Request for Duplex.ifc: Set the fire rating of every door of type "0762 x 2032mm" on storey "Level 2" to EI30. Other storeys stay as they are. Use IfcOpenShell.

First a look at what the model holds.

```python
import ifcopenshell
import ifcopenshell.util.element

model = ifcopenshell.open("Duplex.ifc")
print(model.schema)
storey = next(s for s in model.by_type("IfcBuildingStorey") if s.Name == "Level 2")
doors = [e for e in ifcopenshell.util.element.get_decomposition(storey) if e.is_a("IfcDoor")]
seen = {}
for e in doors:
    element_type = ifcopenshell.util.element.get_type(e)
    key = (element_type.Name if element_type != e and element_type else None, ifcopenshell.util.element.get_pset(e, "Pset_DoorCommon", "FireRating"))
    seen[key] = seen.get(key, 0) + 1
for (name, value), count in sorted(seen.items(), key=str):
    print(count, "x", name, "|", value)
```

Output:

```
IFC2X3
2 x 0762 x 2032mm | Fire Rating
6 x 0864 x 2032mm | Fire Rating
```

```python
import ifcopenshell
import ifcopenshell.api.pset
import ifcopenshell.util.element

model = ifcopenshell.open("Duplex.ifc")

storey = next(s for s in model.by_type("IfcBuildingStorey") if s.Name == "Level 2")
doors = [e for e in ifcopenshell.util.element.get_decomposition(storey) if e.is_a("IfcDoor")]

count = 0
for e in doors:
    element_type = ifcopenshell.util.element.get_type(e)
    if element_type in (None, e) or element_type.Name != "0762 x 2032mm":
        continue
    # add_pset returns the element's existing set when there is one.
    pset = ifcopenshell.api.pset.add_pset(model, product=e, name="Pset_DoorCommon")
    ifcopenshell.api.pset.edit_pset(model, pset=pset, properties={"FireRating": "EI30"})
    count += 1

print(count, "doors updated")

model.write("Duplex_rev.ifc")
```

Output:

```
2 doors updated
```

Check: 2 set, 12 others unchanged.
